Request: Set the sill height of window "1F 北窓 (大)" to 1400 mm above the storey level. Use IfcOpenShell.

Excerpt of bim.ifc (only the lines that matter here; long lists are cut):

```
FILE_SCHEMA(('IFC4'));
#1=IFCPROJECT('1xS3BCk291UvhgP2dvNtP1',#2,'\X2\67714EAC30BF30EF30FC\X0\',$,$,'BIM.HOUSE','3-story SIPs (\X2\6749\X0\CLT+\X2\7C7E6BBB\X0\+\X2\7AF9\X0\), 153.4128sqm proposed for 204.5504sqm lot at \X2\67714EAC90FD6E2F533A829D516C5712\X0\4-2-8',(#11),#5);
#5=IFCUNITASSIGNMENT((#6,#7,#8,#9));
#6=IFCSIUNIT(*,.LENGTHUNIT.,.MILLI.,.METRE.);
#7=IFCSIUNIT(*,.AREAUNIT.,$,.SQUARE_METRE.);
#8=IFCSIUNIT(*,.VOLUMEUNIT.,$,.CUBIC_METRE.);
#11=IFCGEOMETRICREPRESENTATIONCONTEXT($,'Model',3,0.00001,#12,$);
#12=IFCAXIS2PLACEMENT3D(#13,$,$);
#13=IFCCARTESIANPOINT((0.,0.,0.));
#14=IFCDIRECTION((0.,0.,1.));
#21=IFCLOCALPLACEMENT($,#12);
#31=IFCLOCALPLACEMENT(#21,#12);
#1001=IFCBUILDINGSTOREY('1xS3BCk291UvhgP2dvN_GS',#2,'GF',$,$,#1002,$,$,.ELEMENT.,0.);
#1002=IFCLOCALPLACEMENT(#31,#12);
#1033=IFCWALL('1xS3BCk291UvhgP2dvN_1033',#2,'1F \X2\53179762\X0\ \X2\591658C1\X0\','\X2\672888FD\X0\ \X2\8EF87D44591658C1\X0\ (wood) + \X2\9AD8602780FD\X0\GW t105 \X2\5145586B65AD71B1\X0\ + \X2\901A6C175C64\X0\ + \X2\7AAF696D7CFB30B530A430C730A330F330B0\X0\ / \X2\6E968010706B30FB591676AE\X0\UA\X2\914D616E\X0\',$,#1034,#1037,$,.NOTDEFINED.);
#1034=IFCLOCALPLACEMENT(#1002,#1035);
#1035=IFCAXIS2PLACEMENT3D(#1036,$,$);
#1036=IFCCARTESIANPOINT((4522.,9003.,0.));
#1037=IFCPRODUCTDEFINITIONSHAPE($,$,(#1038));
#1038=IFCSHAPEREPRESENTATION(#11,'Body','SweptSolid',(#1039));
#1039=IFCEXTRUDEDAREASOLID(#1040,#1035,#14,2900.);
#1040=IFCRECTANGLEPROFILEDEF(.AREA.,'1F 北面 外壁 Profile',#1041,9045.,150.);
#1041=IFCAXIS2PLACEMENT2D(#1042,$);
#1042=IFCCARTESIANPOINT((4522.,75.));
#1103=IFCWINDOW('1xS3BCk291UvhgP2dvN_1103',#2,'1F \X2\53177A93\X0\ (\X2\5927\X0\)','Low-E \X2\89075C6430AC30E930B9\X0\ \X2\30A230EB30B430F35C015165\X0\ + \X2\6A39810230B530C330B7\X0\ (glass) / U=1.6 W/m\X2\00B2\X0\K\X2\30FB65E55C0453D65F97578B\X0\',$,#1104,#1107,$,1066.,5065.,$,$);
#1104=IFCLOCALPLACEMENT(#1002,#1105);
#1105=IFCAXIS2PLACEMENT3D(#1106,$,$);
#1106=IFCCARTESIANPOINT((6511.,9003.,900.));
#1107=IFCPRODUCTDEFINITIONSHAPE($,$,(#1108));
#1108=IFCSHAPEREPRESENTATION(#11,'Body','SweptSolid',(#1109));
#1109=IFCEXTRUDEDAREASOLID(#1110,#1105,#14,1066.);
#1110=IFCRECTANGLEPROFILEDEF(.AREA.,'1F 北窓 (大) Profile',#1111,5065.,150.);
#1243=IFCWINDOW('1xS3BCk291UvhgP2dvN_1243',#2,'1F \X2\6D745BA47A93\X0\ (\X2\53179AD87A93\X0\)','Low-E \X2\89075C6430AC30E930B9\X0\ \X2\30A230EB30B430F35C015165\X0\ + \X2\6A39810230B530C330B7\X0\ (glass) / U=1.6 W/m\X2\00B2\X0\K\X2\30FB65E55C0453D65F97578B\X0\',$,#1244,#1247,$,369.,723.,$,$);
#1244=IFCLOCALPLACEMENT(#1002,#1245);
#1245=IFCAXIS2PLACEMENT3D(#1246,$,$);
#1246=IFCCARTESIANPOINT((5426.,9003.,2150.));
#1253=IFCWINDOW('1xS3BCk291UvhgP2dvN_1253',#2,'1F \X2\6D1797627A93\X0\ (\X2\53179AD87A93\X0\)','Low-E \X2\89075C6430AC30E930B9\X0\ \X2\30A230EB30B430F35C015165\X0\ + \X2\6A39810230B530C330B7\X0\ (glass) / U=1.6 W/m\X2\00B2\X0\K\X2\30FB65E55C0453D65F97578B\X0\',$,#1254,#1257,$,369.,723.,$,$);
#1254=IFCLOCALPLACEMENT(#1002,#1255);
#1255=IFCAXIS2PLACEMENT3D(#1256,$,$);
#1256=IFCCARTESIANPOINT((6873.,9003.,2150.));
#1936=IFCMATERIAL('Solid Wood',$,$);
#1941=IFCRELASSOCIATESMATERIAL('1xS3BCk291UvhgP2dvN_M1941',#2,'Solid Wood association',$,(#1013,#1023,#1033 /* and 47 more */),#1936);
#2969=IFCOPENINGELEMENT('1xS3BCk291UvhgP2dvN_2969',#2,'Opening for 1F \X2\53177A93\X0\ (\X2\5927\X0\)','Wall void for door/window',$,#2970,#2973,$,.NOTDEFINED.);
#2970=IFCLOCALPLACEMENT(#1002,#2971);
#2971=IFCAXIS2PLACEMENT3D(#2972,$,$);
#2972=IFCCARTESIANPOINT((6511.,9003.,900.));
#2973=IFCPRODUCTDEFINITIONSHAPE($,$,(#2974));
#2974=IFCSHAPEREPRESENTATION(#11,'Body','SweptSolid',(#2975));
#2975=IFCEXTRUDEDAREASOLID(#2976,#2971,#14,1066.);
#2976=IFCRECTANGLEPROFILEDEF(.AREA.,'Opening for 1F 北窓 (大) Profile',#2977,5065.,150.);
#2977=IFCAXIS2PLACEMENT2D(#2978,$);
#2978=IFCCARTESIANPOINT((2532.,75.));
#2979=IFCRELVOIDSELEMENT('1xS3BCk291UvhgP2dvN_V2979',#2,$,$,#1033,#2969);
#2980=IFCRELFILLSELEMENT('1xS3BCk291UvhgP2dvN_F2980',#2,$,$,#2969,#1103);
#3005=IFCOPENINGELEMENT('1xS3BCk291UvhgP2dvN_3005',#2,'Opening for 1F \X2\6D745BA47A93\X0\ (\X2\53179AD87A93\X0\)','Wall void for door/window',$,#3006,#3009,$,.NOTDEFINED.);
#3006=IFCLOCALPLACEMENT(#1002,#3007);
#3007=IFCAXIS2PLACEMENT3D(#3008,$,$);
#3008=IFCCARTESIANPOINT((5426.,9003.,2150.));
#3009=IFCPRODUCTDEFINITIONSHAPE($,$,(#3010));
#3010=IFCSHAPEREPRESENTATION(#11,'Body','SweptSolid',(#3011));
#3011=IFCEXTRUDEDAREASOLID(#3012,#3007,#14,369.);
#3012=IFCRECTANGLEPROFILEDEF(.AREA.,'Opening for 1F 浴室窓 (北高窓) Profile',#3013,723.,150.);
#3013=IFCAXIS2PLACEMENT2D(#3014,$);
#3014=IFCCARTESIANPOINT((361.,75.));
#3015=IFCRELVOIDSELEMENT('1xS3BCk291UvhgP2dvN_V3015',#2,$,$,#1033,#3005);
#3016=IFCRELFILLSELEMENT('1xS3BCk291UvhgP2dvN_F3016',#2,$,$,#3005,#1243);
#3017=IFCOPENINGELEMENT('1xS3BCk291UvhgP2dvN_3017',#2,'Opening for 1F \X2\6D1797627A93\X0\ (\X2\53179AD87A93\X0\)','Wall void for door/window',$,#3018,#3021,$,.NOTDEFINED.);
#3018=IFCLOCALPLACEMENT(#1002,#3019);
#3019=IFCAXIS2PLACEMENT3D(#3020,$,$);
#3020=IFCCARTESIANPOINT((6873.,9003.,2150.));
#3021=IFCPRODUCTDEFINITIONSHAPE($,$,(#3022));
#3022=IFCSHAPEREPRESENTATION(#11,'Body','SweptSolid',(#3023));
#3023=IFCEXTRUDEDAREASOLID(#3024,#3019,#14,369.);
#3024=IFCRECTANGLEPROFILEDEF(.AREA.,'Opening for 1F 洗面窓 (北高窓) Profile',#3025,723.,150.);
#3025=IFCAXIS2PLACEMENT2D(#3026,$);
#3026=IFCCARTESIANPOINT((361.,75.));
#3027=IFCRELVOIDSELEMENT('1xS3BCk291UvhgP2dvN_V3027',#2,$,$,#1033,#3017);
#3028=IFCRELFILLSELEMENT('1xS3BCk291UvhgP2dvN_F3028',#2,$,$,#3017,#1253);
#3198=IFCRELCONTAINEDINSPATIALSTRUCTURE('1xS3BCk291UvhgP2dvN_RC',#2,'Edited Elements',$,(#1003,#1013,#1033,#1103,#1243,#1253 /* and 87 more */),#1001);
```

```python
import numpy as np
import ifcopenshell
import ifcopenshell.api.geometry
import ifcopenshell.geom
import ifcopenshell.util.element
import ifcopenshell.util.placement
import ifcopenshell.util.shape
import ifcopenshell.util.unit

model = ifcopenshell.open("bim.ifc")
unit_scale = ifcopenshell.util.unit.calculate_unit_scale(model)

window = model.by_guid("1xS3BCk291UvhgP2dvN_1103")
opening = window.FillsVoids[0].RelatingOpeningElement
storey = ifcopenshell.util.element.get_container(window, ifc_class="IfcBuildingStorey")
level = ifcopenshell.util.placement.get_local_placement(storey.ObjectPlacement)[2, 3]

# The opening's origin need not be at the sill, so measure its lowest point.
shape = ifcopenshell.geom.create_shape(ifcopenshell.geom.settings(), opening)
bottom = ifcopenshell.util.shape.get_shape_bottom_elevation(shape, shape.geometry) / unit_scale
dz = level + 1.4 / unit_scale - bottom

shift = np.array([0.0, 0.0, dz])
# The window is not placed relative to its opening, so move both.
for product in (opening, window):
    matrix = ifcopenshell.util.placement.get_local_placement(product.ObjectPlacement)
    matrix[:3, 3] += shift
    ifcopenshell.api.geometry.edit_object_placement(model, product=product, matrix=matrix, is_si=False)

print(f"moved by {dz * unit_scale:+.3f} m")

model.write("bim_rev.ifc")
```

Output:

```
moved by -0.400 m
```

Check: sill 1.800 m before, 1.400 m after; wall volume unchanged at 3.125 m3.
